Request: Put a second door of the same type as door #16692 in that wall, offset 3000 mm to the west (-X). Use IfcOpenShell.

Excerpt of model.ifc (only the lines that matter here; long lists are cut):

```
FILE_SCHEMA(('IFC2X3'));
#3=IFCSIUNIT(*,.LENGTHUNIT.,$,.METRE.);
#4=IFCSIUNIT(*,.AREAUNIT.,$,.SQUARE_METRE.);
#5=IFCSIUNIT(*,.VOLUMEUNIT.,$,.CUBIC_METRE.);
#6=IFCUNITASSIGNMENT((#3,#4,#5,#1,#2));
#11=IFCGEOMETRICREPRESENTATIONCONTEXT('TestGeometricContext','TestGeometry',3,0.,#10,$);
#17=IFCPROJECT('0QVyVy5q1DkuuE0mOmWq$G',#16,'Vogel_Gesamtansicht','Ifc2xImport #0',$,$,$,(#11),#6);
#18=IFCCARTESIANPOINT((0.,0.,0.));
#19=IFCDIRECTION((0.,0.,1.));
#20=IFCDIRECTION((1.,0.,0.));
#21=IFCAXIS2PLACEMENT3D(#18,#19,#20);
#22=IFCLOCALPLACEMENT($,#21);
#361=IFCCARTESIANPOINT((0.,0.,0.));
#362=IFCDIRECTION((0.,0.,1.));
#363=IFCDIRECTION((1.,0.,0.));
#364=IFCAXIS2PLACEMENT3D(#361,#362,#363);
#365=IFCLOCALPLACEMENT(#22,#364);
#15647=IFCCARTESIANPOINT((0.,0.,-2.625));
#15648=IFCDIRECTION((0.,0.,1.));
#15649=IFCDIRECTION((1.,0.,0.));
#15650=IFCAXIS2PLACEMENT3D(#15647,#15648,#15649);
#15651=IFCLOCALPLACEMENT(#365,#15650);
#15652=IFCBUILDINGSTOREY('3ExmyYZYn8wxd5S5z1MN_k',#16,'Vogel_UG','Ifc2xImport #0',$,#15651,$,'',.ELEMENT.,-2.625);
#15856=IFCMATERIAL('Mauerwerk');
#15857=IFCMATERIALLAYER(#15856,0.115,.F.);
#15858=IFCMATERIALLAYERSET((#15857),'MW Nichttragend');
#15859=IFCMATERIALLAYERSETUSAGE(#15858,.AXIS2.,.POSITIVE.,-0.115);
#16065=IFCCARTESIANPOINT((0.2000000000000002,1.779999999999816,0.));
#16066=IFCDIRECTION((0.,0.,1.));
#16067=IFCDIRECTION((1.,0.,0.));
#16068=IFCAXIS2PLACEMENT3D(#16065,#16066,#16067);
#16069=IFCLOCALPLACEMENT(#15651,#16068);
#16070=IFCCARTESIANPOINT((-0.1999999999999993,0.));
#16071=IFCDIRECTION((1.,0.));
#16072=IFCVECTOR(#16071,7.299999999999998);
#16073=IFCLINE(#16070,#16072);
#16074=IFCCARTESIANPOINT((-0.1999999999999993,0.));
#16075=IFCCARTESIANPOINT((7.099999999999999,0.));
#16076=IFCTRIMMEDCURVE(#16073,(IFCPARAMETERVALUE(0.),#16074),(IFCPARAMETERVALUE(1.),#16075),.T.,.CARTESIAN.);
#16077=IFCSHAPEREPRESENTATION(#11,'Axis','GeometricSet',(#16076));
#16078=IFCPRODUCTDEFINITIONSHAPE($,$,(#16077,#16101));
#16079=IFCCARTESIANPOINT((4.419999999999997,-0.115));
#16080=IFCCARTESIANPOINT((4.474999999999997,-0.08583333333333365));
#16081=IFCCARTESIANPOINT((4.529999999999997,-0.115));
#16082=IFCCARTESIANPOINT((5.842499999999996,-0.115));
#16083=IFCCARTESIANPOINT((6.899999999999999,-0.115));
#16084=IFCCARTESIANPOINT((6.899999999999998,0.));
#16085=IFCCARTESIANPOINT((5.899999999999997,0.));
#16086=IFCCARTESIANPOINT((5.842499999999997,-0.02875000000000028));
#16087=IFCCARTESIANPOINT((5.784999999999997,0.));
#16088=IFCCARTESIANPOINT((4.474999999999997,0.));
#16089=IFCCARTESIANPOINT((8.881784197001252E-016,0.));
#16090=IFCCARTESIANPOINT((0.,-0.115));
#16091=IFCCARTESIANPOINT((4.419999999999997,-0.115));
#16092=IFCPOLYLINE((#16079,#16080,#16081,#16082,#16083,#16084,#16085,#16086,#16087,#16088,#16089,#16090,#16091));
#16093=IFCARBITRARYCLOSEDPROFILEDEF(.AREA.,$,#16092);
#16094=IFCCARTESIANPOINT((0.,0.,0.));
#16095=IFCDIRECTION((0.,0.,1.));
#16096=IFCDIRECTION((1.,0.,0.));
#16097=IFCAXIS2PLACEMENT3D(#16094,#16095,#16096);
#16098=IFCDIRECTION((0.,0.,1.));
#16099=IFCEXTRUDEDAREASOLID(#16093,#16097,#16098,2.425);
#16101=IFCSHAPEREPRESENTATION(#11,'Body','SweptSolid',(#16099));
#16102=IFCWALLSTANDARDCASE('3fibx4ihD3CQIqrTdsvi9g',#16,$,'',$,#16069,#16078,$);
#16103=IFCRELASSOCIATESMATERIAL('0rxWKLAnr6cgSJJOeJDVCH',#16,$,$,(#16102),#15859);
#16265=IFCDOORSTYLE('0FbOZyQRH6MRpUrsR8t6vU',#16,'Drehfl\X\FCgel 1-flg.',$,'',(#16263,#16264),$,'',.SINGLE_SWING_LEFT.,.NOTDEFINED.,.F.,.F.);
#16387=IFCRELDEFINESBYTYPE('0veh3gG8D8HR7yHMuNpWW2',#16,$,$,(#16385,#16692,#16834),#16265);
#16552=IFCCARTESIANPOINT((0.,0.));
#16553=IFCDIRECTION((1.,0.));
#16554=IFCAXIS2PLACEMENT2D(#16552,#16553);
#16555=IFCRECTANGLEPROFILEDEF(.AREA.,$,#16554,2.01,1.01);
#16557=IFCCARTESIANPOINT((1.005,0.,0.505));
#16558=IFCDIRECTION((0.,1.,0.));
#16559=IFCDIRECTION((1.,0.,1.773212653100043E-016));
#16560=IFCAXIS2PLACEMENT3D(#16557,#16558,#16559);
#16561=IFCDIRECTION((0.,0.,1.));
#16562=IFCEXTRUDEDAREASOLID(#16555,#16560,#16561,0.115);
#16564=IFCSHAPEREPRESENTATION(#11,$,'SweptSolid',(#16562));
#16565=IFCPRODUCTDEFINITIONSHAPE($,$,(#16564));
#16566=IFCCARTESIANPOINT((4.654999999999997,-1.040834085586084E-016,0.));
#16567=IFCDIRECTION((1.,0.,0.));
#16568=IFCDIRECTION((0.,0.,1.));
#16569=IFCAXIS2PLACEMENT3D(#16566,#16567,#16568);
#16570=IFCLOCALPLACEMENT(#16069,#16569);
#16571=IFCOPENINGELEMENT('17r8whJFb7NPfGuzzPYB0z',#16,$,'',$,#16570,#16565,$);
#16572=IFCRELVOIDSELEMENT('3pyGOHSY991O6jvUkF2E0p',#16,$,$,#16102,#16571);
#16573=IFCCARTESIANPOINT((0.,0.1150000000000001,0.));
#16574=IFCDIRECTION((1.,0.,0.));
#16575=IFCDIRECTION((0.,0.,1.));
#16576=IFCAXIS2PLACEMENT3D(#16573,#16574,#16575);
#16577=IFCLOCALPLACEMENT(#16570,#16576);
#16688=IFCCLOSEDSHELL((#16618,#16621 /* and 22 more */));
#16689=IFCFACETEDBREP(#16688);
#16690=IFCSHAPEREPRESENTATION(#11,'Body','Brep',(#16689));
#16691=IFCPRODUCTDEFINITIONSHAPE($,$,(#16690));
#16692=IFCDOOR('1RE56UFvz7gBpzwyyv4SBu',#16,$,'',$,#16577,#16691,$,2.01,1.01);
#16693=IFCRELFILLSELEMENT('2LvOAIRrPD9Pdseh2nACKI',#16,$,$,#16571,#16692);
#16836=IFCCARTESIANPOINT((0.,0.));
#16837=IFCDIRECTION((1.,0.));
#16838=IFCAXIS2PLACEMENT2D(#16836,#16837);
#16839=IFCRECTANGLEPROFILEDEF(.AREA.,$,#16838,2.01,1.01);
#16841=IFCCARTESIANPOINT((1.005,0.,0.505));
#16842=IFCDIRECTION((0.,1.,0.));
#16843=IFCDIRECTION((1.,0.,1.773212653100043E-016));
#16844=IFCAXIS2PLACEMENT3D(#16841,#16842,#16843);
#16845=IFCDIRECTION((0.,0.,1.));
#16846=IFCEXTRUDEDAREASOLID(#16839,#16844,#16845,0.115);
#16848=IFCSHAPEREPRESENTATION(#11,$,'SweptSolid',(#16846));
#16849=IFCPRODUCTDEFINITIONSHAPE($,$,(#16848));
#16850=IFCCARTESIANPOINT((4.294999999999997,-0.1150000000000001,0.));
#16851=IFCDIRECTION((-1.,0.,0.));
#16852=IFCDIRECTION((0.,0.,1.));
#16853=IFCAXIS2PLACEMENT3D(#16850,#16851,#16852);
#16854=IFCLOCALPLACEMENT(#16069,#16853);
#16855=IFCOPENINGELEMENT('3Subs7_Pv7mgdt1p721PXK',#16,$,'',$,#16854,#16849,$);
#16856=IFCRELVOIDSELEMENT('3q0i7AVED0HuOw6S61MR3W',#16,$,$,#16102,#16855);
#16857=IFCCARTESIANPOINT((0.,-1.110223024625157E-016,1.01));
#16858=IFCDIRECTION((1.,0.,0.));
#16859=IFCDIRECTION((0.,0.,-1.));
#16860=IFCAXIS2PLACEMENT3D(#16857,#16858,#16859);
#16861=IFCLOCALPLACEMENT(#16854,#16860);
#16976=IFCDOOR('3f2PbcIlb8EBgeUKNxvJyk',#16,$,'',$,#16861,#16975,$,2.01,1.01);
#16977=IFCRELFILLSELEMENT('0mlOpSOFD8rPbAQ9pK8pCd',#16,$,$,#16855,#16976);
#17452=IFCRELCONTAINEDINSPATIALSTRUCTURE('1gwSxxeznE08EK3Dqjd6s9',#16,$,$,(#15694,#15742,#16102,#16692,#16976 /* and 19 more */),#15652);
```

```python
import ifcopenshell
import ifcopenshell.api.feature
import ifcopenshell.api.geometry
import ifcopenshell.api.root
import ifcopenshell.geom
import ifcopenshell.util.element
import ifcopenshell.util.placement
import ifcopenshell.util.shape
import ifcopenshell.util.unit

model = ifcopenshell.open("model.ifc")
unit_scale = ifcopenshell.util.unit.calculate_unit_scale(model)
settings = ifcopenshell.geom.settings()


def volume(element):
    """Net volume in cubic metres, openings subtracted."""
    shape = ifcopenshell.geom.create_shape(settings, element)
    return ifcopenshell.util.shape.get_volume(shape.geometry)


door = model.by_guid("1RE56UFvz7gBpzwyyv4SBu")
opening = door.FillsVoids[0].RelatingOpeningElement
wall = opening.VoidsElements[0].RelatingBuildingElement
before = volume(wall)
shift = ifcopenshell.util.placement.get_local_placement(wall.ObjectPlacement)[:3, 0] * -3 / unit_scale

# copy_class copies the void relationship, type, container and properties, but no geometry.
new_opening = ifcopenshell.api.root.copy_class(model, product=opening)
new_opening.Representation = ifcopenshell.util.element.copy_deep(
    model, opening.Representation, exclude=["IfcGeometricRepresentationContext", "IfcRepresentationMap"]
)
new_door = ifcopenshell.api.root.copy_class(model, product=door)
new_door.Representation = ifcopenshell.util.element.copy_deep(
    model, door.Representation, exclude=["IfcGeometricRepresentationContext", "IfcRepresentationMap"]
)
fills = ifcopenshell.api.feature.add_filling(model, opening=new_opening, element=new_door)
fills.OwnerHistory = new_door.OwnerHistory  # required in IFC2X3

for old, new in ((opening, new_opening), (door, new_door)):
    matrix = ifcopenshell.util.placement.get_local_placement(old.ObjectPlacement)
    matrix[:3, 3] += shift
    ifcopenshell.api.geometry.edit_object_placement(model, product=new, matrix=matrix, is_si=False)

after = volume(wall)

print(f"wall volume {before:.3f} -> {after:.3f} m3")

model.write("model_rev.ifc")
```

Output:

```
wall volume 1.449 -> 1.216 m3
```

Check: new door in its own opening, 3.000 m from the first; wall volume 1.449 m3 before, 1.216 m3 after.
